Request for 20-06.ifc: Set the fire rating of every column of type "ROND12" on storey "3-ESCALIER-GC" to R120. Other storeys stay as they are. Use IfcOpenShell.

First a look at what the model holds.

```python
import ifcopenshell
import ifcopenshell.util.element

model = ifcopenshell.open("20-06.ifc")
print(model.schema)
storey = next(s for s in model.by_type("IfcBuildingStorey") if s.Name == "3-ESCALIER-GC")
columns = [e for e in ifcopenshell.util.element.get_decomposition(storey) if e.is_a("IfcColumn")]
seen = {}
for e in columns:
    element_type = ifcopenshell.util.element.get_type(e)
    key = (element_type.Name if element_type != e and element_type else None, ifcopenshell.util.element.get_pset(e, "Pset_ColumnCommon", "FireRating"))
    seen[key] = seen.get(key, 0) + 1
for (name, value), count in sorted(seen.items(), key=str):
    print(count, "x", name, "|", value)
```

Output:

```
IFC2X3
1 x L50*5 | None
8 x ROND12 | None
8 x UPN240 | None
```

```python
import ifcopenshell
import ifcopenshell.api.pset
import ifcopenshell.util.element

model = ifcopenshell.open("20-06.ifc")

storey = next(s for s in model.by_type("IfcBuildingStorey") if s.Name == "3-ESCALIER-GC")
columns = [e for e in ifcopenshell.util.element.get_decomposition(storey) if e.is_a("IfcColumn")]

count = 0
for e in columns:
    element_type = ifcopenshell.util.element.get_type(e)
    if element_type in (None, e) or element_type.Name != "ROND12":
        continue
    # add_pset returns the element's existing set when there is one.
    pset = ifcopenshell.api.pset.add_pset(model, product=e, name="Pset_ColumnCommon")
    ifcopenshell.api.pset.edit_pset(model, pset=pset, properties={"FireRating": "R120"})
    count += 1

print(count, "columns updated")

model.write("20-06_rev.ifc")
```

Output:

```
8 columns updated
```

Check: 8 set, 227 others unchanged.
